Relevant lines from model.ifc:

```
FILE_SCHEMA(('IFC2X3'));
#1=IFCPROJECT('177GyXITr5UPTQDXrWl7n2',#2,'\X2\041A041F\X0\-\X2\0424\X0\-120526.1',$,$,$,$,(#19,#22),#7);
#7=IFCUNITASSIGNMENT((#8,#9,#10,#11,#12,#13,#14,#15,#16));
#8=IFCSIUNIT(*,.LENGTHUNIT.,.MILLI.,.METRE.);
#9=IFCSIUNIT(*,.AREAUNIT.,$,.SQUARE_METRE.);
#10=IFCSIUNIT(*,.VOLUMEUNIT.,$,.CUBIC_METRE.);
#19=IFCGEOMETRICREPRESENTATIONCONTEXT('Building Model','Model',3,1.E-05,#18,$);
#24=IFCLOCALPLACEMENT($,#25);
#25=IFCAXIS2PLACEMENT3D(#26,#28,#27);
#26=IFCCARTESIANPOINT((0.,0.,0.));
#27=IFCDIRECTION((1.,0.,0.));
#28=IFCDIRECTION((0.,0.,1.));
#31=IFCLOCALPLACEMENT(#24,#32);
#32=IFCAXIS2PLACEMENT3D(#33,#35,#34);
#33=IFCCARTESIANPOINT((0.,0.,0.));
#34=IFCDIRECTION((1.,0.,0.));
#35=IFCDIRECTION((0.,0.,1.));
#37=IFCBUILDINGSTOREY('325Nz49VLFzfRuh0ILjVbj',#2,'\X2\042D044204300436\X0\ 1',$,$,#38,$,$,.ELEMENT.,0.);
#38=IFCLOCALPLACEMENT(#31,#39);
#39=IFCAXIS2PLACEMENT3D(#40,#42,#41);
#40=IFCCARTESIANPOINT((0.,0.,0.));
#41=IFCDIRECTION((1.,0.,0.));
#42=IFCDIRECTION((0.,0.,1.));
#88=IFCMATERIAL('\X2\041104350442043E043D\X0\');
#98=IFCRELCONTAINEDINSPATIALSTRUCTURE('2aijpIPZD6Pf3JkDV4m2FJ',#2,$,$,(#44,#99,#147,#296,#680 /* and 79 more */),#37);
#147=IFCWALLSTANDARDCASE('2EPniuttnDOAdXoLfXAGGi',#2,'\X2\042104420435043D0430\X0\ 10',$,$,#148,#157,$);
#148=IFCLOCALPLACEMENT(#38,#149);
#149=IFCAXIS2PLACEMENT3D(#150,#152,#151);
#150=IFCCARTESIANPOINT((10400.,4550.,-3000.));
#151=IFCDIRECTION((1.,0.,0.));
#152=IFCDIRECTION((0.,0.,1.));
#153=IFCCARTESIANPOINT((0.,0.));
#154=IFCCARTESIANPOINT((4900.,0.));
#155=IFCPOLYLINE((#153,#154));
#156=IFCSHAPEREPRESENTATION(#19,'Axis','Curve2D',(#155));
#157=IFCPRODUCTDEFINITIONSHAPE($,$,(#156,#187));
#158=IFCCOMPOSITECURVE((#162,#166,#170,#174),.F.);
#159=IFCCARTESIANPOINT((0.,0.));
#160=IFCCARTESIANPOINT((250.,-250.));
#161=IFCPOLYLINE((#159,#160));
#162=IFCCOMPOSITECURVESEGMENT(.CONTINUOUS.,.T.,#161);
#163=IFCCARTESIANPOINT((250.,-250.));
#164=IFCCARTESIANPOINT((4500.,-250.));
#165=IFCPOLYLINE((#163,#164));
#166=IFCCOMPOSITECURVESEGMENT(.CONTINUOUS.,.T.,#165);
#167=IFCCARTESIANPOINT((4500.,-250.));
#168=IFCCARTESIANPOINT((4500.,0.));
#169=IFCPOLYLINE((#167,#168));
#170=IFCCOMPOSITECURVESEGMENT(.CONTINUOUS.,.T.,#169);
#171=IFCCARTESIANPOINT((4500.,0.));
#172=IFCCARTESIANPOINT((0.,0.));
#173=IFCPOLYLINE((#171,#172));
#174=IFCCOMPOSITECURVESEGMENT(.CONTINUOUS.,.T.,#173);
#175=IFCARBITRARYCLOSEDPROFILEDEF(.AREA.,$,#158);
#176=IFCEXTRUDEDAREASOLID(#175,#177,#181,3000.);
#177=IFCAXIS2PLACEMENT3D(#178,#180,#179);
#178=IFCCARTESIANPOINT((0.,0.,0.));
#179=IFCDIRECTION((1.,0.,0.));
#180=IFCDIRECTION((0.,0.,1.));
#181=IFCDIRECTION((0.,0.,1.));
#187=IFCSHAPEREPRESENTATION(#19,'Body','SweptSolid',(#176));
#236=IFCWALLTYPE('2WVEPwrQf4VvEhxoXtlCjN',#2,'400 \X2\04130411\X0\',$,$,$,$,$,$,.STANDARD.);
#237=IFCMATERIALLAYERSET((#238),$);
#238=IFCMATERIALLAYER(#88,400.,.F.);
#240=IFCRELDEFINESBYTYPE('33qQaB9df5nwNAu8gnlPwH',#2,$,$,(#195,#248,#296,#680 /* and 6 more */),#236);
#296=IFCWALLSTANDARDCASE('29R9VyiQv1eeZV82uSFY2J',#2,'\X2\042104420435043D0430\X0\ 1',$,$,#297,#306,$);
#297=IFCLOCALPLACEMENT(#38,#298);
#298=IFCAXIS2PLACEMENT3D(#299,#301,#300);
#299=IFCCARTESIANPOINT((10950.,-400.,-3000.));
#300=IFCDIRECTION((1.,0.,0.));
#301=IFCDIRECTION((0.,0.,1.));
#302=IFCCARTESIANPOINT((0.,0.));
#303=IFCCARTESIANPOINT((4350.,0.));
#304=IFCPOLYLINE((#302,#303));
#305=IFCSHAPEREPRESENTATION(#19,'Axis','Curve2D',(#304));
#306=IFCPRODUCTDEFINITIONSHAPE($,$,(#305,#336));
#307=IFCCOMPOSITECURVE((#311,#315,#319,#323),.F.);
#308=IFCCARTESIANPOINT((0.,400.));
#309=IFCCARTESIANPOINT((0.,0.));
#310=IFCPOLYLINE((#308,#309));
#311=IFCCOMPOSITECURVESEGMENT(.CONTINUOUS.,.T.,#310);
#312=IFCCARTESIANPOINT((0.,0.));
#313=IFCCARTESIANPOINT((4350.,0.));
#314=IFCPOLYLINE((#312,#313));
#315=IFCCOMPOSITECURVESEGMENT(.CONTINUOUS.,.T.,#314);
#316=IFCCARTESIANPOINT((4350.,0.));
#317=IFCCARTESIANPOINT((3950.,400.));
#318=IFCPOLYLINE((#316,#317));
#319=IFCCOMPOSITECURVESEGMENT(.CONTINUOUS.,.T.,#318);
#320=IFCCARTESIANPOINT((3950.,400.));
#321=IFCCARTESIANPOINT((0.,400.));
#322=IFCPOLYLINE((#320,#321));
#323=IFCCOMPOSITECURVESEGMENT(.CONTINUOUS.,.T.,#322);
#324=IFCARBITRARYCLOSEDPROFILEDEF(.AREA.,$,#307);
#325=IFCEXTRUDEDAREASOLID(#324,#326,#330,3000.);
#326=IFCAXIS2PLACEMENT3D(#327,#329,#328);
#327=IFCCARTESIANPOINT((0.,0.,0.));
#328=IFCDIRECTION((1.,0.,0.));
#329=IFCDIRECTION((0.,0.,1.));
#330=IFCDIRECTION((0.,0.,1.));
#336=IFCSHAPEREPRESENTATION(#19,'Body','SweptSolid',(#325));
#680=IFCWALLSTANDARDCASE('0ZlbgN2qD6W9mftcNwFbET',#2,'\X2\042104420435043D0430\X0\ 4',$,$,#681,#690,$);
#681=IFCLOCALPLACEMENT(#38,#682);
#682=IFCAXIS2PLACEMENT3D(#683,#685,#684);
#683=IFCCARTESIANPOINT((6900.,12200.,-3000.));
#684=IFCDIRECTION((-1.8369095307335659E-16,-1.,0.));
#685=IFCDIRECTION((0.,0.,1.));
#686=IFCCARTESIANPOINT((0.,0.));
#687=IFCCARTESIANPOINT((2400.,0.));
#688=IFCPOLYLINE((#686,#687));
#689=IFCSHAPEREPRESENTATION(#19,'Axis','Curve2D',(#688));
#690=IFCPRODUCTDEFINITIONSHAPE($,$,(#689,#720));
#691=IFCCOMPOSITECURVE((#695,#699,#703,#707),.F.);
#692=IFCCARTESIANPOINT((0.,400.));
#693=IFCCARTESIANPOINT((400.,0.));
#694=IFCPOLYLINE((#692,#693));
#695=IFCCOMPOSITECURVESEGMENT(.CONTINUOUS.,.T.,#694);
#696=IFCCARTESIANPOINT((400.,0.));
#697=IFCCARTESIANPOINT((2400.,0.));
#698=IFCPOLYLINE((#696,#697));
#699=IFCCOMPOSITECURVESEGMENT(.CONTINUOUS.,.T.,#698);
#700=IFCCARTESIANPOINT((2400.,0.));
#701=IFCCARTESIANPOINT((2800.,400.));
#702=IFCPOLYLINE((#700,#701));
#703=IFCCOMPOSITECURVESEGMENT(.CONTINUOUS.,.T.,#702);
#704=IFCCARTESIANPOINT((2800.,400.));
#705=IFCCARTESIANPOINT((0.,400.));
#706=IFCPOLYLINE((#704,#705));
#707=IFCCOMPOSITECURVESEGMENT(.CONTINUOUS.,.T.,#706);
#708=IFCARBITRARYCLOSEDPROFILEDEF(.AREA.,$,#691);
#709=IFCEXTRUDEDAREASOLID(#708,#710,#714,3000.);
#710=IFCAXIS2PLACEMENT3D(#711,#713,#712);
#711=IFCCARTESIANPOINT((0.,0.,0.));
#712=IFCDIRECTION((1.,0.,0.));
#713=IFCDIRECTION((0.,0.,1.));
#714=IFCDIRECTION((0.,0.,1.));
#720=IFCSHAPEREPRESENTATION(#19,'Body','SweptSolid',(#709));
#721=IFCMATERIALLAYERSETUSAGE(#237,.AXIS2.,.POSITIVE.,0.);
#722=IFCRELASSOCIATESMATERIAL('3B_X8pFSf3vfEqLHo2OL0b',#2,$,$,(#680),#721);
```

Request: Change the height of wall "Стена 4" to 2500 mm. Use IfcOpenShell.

```python
import ifcopenshell
import ifcopenshell.geom
import ifcopenshell.util.shape
import ifcopenshell.util.unit

model = ifcopenshell.open("model.ifc")
unit_scale = ifcopenshell.util.unit.calculate_unit_scale(model)
settings = ifcopenshell.geom.settings()


def volume(element):
    """Net volume in cubic metres, openings subtracted."""
    shape = ifcopenshell.geom.create_shape(settings, element)
    return ifcopenshell.util.shape.get_volume(shape.geometry)


wall = model.by_id(680)
before = volume(wall)

body = next(r for r in wall.Representation.Representations if r.RepresentationIdentifier == "Body")
solid = body.Items[0]
old_height = solid.Depth
solid.Depth = 2.5 / unit_scale
after = volume(wall)

print(f"height {old_height:g} -> {solid.Depth:g}, volume {before:.3f} -> {after:.3f} m3")

model.write("model_v2.ifc")
```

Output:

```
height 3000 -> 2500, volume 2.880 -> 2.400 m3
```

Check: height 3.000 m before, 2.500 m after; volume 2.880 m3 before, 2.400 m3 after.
